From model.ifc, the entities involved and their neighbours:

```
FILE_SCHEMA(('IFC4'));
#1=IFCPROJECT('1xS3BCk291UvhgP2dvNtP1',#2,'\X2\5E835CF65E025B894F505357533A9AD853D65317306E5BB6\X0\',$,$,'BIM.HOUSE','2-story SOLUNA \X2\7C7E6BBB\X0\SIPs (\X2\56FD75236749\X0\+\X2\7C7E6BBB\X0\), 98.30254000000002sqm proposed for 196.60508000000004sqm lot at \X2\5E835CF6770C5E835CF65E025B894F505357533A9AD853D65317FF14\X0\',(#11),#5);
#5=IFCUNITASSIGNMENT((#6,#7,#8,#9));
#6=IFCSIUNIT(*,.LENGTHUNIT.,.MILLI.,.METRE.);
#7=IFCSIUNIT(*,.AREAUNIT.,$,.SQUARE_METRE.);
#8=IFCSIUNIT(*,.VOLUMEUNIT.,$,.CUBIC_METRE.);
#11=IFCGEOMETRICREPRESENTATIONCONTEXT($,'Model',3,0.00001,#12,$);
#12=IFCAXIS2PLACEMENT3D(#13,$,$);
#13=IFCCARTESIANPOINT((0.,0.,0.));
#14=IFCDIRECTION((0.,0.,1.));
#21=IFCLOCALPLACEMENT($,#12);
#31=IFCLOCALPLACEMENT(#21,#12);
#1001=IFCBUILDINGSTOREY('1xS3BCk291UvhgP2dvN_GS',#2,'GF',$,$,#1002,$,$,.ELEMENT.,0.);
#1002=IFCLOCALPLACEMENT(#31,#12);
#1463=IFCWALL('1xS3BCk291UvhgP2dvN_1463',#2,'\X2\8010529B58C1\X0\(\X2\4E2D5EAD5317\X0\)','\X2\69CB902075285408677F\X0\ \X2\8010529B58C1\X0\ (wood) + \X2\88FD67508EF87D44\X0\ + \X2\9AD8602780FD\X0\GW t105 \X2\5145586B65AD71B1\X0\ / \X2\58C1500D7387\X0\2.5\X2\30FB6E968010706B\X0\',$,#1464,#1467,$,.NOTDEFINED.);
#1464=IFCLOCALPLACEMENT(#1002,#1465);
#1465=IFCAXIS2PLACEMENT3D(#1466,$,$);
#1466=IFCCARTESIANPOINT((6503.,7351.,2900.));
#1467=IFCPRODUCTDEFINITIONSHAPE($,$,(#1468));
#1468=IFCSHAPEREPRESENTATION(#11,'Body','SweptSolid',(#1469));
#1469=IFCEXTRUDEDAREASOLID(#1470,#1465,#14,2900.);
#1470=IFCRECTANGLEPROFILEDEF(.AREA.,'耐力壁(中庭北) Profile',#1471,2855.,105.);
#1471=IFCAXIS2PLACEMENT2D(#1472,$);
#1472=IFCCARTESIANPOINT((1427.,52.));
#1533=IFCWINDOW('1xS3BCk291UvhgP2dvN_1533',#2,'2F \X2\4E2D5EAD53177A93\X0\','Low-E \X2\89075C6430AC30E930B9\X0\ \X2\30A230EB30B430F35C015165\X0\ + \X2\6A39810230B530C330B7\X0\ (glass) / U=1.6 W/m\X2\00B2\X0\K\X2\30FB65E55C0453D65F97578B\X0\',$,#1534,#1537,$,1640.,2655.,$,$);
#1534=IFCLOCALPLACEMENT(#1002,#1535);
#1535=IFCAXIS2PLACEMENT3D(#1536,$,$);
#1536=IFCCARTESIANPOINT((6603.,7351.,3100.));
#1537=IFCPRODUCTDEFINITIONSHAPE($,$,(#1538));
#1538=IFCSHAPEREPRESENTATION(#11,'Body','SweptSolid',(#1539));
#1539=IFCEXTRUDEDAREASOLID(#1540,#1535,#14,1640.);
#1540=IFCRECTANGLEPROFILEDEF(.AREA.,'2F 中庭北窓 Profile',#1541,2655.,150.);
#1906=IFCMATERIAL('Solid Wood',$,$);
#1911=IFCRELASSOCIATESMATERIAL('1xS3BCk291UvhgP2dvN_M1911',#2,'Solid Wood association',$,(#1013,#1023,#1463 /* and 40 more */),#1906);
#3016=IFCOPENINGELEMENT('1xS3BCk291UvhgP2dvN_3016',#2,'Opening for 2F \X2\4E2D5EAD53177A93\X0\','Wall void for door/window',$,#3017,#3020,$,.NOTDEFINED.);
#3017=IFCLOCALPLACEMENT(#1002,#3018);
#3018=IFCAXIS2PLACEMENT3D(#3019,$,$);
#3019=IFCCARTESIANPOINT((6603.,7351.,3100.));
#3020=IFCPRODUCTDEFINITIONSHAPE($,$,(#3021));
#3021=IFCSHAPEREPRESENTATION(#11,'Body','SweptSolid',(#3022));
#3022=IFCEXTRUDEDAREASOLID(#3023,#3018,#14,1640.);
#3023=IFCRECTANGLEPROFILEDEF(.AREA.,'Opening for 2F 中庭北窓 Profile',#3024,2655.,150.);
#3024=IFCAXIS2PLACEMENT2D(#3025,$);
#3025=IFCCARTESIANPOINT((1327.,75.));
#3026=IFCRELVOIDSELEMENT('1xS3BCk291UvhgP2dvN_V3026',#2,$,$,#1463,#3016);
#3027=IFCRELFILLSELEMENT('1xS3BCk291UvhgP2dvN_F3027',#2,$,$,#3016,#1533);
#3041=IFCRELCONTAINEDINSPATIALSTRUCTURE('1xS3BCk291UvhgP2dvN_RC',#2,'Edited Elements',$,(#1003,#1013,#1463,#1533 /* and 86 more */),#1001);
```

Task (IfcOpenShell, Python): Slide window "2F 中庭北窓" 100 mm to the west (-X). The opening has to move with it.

```python
import ifcopenshell
import ifcopenshell.api.geometry
import ifcopenshell.util.placement

model = ifcopenshell.open("model.ifc")

window = model.by_id(1533)
opening = window.FillsVoids[0].RelatingOpeningElement
wall = opening.VoidsElements[0].RelatingBuildingElement

wall_matrix = ifcopenshell.util.placement.get_local_placement(wall.ObjectPlacement)
shift = wall_matrix[:3, 0] * -100.0
before = ifcopenshell.util.placement.get_local_placement(window.ObjectPlacement)[:3, 3].copy()

# The window is not placed relative to its opening, so move both.
for product in (opening, window):
    matrix = ifcopenshell.util.placement.get_local_placement(product.ObjectPlacement)
    matrix[:3, 3] += shift
    ifcopenshell.api.geometry.edit_object_placement(model, product=product, matrix=matrix, is_si=False)

after = ifcopenshell.util.placement.get_local_placement(window.ObjectPlacement)[:3, 3]
print("window moved by", (after - before).round(3) + 0.0)

model.write("model_edited.ifc")
```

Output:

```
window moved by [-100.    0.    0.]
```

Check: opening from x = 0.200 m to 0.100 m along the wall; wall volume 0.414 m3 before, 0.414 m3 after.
